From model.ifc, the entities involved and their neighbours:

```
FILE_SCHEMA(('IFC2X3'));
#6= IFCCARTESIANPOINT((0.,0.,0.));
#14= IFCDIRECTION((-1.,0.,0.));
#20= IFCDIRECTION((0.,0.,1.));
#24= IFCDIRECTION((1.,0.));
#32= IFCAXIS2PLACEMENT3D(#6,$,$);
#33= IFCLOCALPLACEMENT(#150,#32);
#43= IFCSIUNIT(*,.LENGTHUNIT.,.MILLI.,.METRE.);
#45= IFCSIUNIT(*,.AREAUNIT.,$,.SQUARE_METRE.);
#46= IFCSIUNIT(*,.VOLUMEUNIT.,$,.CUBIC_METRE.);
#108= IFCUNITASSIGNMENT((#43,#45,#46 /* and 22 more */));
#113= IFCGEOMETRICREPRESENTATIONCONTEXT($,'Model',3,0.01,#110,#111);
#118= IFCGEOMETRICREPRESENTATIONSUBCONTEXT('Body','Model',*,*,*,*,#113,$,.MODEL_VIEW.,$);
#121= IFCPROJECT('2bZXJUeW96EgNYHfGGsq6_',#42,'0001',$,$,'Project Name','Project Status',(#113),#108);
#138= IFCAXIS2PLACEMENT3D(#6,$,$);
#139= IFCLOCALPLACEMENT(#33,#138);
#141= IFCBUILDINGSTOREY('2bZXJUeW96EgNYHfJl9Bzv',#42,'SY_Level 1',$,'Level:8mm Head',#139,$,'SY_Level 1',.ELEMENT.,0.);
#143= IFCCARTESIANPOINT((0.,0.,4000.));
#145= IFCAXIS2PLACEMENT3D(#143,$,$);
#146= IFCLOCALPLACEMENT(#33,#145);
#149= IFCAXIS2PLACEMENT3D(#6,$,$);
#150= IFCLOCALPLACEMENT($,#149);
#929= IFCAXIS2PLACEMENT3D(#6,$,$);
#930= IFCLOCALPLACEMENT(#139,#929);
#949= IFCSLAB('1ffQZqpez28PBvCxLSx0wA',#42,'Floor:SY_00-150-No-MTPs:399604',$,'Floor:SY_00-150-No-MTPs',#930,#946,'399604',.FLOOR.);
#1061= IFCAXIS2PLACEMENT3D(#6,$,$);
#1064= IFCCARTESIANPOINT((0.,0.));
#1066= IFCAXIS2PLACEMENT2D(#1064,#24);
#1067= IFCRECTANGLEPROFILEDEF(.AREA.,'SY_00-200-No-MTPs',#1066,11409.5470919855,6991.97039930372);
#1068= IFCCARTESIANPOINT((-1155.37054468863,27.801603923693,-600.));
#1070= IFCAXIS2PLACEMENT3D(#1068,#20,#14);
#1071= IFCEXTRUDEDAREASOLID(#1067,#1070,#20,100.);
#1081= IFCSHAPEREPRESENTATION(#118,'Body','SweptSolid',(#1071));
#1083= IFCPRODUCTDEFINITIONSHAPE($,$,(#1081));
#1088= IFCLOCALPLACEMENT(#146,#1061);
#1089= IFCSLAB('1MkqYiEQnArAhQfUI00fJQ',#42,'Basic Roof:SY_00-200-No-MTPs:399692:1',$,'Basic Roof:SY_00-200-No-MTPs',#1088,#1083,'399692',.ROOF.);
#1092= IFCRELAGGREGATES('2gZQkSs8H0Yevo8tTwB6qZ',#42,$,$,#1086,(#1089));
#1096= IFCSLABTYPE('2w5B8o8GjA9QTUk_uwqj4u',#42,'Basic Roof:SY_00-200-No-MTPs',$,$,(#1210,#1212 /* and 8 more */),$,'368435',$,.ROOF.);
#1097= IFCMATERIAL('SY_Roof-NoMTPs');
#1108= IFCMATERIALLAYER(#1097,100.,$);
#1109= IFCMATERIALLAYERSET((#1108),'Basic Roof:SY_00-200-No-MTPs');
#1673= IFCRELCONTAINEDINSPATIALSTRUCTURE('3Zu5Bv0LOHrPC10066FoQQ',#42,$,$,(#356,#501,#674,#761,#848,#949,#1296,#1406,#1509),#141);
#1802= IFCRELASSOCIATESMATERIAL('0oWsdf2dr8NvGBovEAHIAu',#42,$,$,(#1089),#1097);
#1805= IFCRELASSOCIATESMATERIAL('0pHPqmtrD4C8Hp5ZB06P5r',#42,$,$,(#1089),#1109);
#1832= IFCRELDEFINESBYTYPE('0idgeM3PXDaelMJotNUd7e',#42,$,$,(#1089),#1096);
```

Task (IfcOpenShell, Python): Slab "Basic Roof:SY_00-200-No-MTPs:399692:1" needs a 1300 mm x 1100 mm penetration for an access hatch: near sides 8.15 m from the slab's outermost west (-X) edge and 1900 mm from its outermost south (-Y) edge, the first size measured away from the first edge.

```python
import numpy as np
import ifcopenshell
import ifcopenshell.api.feature
import ifcopenshell.api.geometry
import ifcopenshell.api.root
import ifcopenshell.geom
import ifcopenshell.util.placement
import ifcopenshell.util.representation
import ifcopenshell.util.shape
import ifcopenshell.util.unit

model = ifcopenshell.open("model.ifc")
unit_scale = ifcopenshell.util.unit.calculate_unit_scale(model)
settings = ifcopenshell.geom.settings()


def volume(element):
    """Net volume in cubic metres, openings subtracted."""
    shape = ifcopenshell.geom.create_shape(settings, element)
    return ifcopenshell.util.shape.get_volume(shape.geometry)


slab = model.by_guid("1MkqYiEQnArAhQfUI00fJQ")
before = volume(slab)

# Extent in the slab's own axes, in metres. The edges named are its -X and -Y sides.
slab_shape = ifcopenshell.geom.create_shape(settings, slab)
vertices = ifcopenshell.util.shape.get_vertices(slab_shape.geometry)
x_min, y_min, bottom = vertices.min(axis=0)
top = vertices[:, 2].max()

opening = ifcopenshell.api.root.create_entity(model, ifc_class="IfcOpeningElement", name="Access hatch opening")
context = ifcopenshell.util.representation.get_context(model, "Model", "Body", "MODEL_VIEW")
width, depth = 1.3, 1.1
outline = [(0.0, 0.0), (width, 0.0), (width, depth), (0.0, depth), (0.0, 0.0)]
# Overshoot both faces by 50 mm so the cut is clean.
shape = ifcopenshell.api.geometry.add_slab_representation(
    model, context=context, depth=top - bottom + 0.1, polyline=outline
)
ifcopenshell.api.geometry.assign_representation(model, product=opening, representation=shape)

matrix = ifcopenshell.util.placement.get_local_placement(slab.ObjectPlacement)
matrix[:, 3] = matrix @ np.append(np.array([x_min + 8.15, y_min + 1.9, bottom - 0.05]) / unit_scale, 1.0)
ifcopenshell.api.geometry.edit_object_placement(model, product=opening, matrix=matrix, is_si=False)
ifcopenshell.api.feature.add_feature(model, feature=opening, element=slab)

after = volume(slab)

print(f"slab volume {before:.3f} -> {after:.3f} m3")

model.write("model_edited.ifc")
```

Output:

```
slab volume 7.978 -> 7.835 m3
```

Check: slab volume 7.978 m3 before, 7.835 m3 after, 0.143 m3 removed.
